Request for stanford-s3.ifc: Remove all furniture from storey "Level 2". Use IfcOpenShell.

First a look at what the model holds.

```python
import ifcopenshell
import ifcopenshell.util.element

model = ifcopenshell.open("stanford-s3.ifc")
print(model.schema)
storey = next(s for s in model.by_type("IfcBuildingStorey") if s.Name == "Level 2")
furniture = [e for e in ifcopenshell.util.element.get_decomposition(storey) if e.is_a("IfcFurnishingElement")]
seen = {}
for e in furniture:
    element_type = ifcopenshell.util.element.get_type(e)
    name = element_type.Name if element_type not in (None, e) else None
    seen[name] = seen.get(name, 0) + 1
for name, count in sorted(seen.items(), key=str):
    print(count, "x", name)
```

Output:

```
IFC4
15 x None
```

```python
import ifcopenshell
import ifcopenshell.api.root
import ifcopenshell.util.element

model = ifcopenshell.open("stanford-s3.ifc")

storey = next(s for s in model.by_type("IfcBuildingStorey") if s.Name == "Level 2")
furniture = [e for e in ifcopenshell.util.element.get_decomposition(storey) if e.is_a("IfcFurnishingElement")]

for e in furniture:
    ifcopenshell.api.root.remove_product(model, product=e)
print(len(furniture), "removed")

model.write("stanford-s3_updated.ifc")
```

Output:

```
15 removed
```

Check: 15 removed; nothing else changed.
